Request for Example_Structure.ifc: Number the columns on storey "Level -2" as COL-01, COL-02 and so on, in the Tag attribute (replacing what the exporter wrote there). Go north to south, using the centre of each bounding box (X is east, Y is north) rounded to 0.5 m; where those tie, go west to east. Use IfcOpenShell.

First a look at what the model holds.

```python
import ifcopenshell
import ifcopenshell.util.element
import ifcopenshell.util.placement

model = ifcopenshell.open("Example_Structure.ifc")
print(model.schema)
storey = next(s for s in model.by_type("IfcBuildingStorey") if s.Name == "Level -2")
columns = [e for e in ifcopenshell.util.element.get_decomposition(storey) if e.is_a("IfcColumn")]
for e in sorted(columns, key=lambda e: e.id()):
    origin = ifcopenshell.util.placement.get_local_placement(e.ObjectPlacement)[:3, 3]
    print(e.id(), e.Tag, e.Name, origin.round(2) + 0.0, sep=" | ")
```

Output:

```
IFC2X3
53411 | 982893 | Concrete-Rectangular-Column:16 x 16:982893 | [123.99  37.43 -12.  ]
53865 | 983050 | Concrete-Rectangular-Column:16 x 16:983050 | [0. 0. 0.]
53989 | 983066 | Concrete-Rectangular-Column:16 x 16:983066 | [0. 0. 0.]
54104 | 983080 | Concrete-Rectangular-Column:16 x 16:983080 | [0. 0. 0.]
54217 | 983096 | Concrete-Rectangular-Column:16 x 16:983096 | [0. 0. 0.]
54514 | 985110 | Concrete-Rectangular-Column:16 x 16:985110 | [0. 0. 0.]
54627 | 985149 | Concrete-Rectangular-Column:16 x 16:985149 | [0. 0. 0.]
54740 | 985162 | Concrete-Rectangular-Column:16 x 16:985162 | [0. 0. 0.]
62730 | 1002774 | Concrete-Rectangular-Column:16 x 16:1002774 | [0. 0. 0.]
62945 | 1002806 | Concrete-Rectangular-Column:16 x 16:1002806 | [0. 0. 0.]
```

```python
import ifcopenshell
import ifcopenshell.geom
import ifcopenshell.util.element
import ifcopenshell.util.shape

model = ifcopenshell.open("Example_Structure.ifc")
settings = ifcopenshell.geom.settings()
settings.set("use-world-coords", True)


def centre(element):
    shape = ifcopenshell.geom.create_shape(settings, element)
    return ifcopenshell.util.shape.get_bbox_centroid(shape.geometry)


storey = next(s for s in model.by_type("IfcBuildingStorey") if s.Name == "Level -2")
columns = [e for e in ifcopenshell.util.element.get_decomposition(storey) if e.is_a("IfcColumn")]

# Insertion points can sit at a corner or the storey origin, so sort by the geometry (in metres).
centres = {e: centre(e) for e in columns}
columns.sort(key=lambda e: (-round(centres[e][1] / 0.5), centres[e][0]))

for i, e in enumerate(columns, start=1):
    number = f"COL-{i:02d}"
    e.Tag = number
    print(e.id(), number)

model.write("Example_Structure_edited.ifc")
```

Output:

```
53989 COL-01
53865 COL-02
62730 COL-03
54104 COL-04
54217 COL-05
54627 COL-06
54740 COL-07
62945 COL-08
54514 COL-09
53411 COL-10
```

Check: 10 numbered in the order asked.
